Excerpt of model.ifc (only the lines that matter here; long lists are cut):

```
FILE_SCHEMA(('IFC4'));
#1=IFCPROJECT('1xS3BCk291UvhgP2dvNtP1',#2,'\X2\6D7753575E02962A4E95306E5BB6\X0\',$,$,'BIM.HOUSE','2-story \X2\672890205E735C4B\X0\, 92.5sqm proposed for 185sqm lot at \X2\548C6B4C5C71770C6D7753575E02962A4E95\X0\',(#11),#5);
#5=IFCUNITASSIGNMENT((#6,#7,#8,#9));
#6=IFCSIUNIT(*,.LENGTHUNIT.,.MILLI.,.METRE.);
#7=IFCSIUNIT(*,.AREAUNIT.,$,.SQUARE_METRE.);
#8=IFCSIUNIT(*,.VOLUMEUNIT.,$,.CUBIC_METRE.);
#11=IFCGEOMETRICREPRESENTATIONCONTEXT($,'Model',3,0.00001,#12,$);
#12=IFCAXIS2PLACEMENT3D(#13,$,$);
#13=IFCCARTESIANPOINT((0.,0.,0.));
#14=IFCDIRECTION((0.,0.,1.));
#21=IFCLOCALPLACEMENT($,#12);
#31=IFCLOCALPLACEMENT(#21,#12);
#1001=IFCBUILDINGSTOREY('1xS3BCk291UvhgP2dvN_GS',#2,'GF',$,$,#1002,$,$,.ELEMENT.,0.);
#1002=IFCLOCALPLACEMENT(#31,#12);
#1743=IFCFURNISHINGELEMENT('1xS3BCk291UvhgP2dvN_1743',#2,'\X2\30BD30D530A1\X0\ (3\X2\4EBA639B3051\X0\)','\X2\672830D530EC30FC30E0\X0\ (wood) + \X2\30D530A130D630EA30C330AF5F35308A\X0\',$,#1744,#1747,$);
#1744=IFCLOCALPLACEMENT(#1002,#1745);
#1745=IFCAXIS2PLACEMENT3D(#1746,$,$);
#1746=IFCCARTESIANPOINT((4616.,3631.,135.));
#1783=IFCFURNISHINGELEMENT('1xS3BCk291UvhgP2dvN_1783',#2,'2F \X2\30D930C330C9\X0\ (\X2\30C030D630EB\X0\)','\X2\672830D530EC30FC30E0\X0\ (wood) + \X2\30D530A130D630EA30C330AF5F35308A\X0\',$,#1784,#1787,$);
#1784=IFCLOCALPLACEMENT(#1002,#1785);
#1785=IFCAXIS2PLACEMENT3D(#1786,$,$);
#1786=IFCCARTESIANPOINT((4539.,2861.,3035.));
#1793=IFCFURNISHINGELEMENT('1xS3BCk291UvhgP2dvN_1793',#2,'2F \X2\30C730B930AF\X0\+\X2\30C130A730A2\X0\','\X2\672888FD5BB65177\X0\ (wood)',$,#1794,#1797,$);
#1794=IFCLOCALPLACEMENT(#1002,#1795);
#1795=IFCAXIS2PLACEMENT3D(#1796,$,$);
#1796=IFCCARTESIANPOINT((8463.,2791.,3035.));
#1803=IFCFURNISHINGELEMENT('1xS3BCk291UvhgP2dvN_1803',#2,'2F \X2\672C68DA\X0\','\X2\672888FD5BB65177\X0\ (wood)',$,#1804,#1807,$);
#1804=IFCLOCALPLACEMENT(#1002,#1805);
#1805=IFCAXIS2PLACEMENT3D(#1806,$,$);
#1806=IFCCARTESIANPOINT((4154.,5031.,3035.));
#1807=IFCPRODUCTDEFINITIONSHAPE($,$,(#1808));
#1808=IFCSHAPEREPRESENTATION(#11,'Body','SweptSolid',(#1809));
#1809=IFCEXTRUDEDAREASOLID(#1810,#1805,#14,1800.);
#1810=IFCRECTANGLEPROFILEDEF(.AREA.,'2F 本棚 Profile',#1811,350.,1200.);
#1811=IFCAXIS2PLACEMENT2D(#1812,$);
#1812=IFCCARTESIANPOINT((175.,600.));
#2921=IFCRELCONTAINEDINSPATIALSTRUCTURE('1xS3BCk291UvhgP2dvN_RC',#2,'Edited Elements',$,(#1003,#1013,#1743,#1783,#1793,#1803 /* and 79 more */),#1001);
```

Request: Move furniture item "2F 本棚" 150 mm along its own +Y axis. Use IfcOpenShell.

```python
import ifcopenshell
import ifcopenshell.api.geometry
import ifcopenshell.util.placement
import ifcopenshell.util.unit

model = ifcopenshell.open("model.ifc")
unit_scale = ifcopenshell.util.unit.calculate_unit_scale(model)

item = model.by_guid("1xS3BCk291UvhgP2dvN_1803")
matrix = ifcopenshell.util.placement.get_local_placement(item.ObjectPlacement)
matrix[:3, 3] += matrix[:3, 1] * 0.15 / unit_scale
ifcopenshell.api.geometry.edit_object_placement(model, product=item, matrix=matrix, is_si=False)

print(ifcopenshell.util.placement.get_local_placement(item.ObjectPlacement).round(3) + 0.0)

model.write("model_rev.ifc")
```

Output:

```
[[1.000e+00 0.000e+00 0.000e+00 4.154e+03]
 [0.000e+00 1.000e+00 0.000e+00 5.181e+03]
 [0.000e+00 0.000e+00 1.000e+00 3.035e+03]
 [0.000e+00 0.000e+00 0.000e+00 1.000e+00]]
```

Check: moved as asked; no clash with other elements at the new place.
